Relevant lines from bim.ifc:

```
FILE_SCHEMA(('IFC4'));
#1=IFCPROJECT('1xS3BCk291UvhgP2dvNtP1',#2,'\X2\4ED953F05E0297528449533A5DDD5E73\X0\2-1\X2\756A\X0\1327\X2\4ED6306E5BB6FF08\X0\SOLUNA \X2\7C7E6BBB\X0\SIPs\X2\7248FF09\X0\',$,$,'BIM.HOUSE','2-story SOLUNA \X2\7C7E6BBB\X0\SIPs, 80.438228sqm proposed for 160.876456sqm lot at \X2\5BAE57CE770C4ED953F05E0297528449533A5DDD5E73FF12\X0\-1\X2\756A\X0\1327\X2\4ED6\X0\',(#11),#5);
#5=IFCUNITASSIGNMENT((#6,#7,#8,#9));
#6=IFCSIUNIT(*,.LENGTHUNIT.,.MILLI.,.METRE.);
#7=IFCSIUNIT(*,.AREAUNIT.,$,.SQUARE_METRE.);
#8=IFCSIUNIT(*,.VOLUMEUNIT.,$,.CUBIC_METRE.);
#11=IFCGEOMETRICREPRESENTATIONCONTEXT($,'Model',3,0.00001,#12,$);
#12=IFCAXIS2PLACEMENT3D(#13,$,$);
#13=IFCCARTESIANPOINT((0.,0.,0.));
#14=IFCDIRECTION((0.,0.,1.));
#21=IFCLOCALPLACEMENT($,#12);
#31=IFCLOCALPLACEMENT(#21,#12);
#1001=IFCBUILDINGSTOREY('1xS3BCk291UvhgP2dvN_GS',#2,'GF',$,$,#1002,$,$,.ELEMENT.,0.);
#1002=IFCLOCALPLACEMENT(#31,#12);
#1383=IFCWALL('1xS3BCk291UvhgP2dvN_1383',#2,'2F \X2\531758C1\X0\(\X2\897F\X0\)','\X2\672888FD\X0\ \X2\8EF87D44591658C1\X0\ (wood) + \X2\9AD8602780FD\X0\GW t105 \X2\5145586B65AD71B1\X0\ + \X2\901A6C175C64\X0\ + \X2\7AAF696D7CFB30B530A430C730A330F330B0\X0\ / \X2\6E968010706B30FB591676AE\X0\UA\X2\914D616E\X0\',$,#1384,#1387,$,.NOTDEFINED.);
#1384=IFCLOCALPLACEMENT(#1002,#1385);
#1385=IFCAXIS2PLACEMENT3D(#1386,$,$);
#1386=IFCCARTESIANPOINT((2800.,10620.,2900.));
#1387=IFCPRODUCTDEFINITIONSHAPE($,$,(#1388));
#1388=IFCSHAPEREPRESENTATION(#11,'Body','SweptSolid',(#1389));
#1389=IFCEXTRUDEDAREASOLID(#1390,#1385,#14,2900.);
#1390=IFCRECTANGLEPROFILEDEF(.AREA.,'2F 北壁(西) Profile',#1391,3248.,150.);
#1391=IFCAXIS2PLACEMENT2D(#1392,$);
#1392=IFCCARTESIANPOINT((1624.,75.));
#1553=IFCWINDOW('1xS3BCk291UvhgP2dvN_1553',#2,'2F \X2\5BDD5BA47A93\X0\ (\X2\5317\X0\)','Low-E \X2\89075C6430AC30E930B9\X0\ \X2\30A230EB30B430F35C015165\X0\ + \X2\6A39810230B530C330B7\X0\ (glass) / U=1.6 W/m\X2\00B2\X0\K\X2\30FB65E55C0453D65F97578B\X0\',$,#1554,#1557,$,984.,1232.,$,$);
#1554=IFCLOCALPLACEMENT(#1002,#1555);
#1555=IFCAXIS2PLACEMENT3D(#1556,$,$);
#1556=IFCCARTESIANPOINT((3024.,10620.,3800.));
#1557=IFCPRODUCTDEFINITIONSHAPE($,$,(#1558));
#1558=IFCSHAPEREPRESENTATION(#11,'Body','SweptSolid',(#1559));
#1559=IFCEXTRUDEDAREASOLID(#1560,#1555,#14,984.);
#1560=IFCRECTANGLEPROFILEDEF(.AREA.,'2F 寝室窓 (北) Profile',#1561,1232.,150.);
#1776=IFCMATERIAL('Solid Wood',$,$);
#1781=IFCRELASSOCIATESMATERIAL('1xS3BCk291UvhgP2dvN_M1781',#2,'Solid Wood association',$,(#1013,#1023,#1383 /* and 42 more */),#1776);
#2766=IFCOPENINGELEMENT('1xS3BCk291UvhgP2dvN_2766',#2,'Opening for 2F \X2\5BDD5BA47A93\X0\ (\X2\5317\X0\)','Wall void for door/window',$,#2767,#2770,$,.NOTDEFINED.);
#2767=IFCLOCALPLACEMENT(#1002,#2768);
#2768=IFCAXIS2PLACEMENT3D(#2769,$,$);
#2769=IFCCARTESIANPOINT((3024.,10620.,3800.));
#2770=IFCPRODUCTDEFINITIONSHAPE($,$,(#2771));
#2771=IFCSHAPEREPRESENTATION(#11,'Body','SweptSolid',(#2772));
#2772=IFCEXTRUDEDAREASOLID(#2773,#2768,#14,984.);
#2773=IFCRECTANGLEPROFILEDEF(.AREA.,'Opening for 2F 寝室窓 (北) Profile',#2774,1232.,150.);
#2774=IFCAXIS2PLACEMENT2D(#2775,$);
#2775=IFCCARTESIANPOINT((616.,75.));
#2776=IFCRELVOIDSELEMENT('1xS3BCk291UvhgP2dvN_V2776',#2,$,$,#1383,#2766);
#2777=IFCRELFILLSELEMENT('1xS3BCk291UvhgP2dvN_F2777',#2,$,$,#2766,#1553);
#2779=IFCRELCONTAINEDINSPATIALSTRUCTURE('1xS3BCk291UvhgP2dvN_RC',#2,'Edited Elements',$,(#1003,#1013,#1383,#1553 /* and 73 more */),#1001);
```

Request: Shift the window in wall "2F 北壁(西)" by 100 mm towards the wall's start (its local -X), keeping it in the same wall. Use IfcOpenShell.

```python
import ifcopenshell
import ifcopenshell.api.geometry
import ifcopenshell.util.placement
import ifcopenshell.util.unit

model = ifcopenshell.open("bim.ifc")
unit_scale = ifcopenshell.util.unit.calculate_unit_scale(model)

window = model.by_guid("1xS3BCk291UvhgP2dvN_1553")
opening = window.FillsVoids[0].RelatingOpeningElement
wall = opening.VoidsElements[0].RelatingBuildingElement

wall_matrix = ifcopenshell.util.placement.get_local_placement(wall.ObjectPlacement)
shift = wall_matrix[:3, 0] * -0.1 / unit_scale
before = ifcopenshell.util.placement.get_local_placement(window.ObjectPlacement)[:3, 3].copy()

# The window is not placed relative to its opening, so move both.
for product in (opening, window):
    matrix = ifcopenshell.util.placement.get_local_placement(product.ObjectPlacement)
    matrix[:3, 3] += shift
    ifcopenshell.api.geometry.edit_object_placement(model, product=product, matrix=matrix, is_si=False)

after = ifcopenshell.util.placement.get_local_placement(window.ObjectPlacement)[:3, 3]
print("window moved by", (after - before).round(3) + 0.0)

model.write("bim_v2.ifc")
```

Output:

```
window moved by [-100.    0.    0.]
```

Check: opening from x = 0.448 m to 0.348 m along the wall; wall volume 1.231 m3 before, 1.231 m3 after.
